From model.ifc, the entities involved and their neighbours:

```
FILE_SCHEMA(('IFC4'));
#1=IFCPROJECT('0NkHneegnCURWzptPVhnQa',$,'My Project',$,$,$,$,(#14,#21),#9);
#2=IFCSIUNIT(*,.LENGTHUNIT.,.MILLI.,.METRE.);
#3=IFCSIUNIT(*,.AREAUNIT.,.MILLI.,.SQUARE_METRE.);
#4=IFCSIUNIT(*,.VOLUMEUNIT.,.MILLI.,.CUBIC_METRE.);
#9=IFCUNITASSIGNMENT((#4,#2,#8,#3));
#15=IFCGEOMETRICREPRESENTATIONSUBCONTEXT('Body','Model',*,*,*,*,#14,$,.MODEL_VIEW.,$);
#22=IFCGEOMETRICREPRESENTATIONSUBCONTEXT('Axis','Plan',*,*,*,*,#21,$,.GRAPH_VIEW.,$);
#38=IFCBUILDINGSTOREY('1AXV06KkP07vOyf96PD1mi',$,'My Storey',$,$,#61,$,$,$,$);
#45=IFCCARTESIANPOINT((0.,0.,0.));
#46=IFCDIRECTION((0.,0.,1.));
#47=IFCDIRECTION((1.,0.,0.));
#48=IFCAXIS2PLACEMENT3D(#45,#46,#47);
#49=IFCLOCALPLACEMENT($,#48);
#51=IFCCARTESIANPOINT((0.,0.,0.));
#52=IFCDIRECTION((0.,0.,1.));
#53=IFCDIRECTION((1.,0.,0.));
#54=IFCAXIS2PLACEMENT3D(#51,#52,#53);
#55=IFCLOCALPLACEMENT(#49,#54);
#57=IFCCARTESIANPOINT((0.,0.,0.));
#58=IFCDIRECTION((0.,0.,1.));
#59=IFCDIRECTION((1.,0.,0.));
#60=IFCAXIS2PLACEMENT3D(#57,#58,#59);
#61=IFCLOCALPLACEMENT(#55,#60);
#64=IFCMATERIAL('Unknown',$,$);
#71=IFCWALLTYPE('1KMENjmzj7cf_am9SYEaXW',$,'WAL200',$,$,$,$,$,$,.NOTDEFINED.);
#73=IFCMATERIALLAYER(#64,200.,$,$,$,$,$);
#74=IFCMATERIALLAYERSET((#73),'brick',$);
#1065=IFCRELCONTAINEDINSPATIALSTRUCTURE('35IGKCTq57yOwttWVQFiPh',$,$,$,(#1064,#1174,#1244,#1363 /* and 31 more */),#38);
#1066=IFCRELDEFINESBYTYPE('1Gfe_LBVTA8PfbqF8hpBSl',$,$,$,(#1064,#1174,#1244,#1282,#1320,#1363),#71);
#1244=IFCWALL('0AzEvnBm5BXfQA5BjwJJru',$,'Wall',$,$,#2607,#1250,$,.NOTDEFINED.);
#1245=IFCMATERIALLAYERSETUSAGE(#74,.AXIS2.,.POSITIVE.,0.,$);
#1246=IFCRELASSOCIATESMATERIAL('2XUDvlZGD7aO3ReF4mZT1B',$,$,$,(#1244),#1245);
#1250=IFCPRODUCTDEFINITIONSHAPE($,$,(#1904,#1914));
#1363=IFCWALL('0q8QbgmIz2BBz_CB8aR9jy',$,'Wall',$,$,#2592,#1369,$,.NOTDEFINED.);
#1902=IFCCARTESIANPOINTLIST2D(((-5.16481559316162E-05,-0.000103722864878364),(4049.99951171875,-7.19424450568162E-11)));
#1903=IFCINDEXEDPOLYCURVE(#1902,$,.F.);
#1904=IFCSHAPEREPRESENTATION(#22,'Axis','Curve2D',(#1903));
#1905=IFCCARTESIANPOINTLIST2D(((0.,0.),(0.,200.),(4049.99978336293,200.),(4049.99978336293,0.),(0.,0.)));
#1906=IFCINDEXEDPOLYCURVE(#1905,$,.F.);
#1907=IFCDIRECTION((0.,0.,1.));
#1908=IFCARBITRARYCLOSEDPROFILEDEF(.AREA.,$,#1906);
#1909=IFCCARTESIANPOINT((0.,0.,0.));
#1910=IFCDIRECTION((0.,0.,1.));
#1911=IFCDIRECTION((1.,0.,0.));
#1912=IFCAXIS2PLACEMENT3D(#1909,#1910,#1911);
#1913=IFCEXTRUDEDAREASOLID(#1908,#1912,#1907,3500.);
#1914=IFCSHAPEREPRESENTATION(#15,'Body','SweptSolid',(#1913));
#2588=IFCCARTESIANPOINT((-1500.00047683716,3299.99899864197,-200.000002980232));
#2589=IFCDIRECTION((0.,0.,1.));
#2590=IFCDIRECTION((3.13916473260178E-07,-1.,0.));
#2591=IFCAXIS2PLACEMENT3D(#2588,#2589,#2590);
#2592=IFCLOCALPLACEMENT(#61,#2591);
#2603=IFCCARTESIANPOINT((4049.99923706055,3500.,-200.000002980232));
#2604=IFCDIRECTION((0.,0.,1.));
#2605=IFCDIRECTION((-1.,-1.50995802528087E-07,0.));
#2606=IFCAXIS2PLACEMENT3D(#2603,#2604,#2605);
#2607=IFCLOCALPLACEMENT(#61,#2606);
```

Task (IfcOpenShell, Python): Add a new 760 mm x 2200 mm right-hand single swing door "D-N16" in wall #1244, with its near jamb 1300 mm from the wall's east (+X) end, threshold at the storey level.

```python
import numpy as np
import ifcopenshell
import ifcopenshell.api.feature
import ifcopenshell.api.geometry
import ifcopenshell.api.root
import ifcopenshell.api.spatial
import ifcopenshell.geom
import ifcopenshell.util.element
import ifcopenshell.util.placement
import ifcopenshell.util.representation
import ifcopenshell.util.shape
import ifcopenshell.util.unit

model = ifcopenshell.open("model.ifc")
unit_scale = ifcopenshell.util.unit.calculate_unit_scale(model)
settings = ifcopenshell.geom.settings()


def volume(element):
    """Net volume in cubic metres, openings subtracted."""
    shape = ifcopenshell.geom.create_shape(settings, element)
    return ifcopenshell.util.shape.get_volume(shape.geometry)


wall = model.by_guid("0AzEvnBm5BXfQA5BjwJJru")
storey = ifcopenshell.util.element.get_container(wall, ifc_class="IfcBuildingStorey")
context = ifcopenshell.util.representation.get_context(model, "Model", "Body", "MODEL_VIEW")
before = volume(wall)

width, height, from_end, sill = 0.76, 2.2, 1.3, 0.0  # metres

# The wall runs along its own X axis, and the end named is its -X end.
wall_shape = ifcopenshell.geom.create_shape(settings, wall)
x, y, z = ifcopenshell.util.shape.get_vertices(wall_shape.geometry).T
start = x.min() + from_end
face, thickness = float(y.min()), float(y.max() - y.min())
wall_matrix = ifcopenshell.util.placement.get_local_placement(wall.ObjectPlacement)
level = ifcopenshell.util.placement.get_local_placement(storey.ObjectPlacement)[2, 3]


def in_wall(x, y):
    """Placement at x, y metres in the wall's axes, at sill height."""
    matrix = wall_matrix.copy()
    matrix[:, 3] = wall_matrix @ np.array([x / unit_scale, y / unit_scale, 0.0, 1.0])
    matrix[2, 3] = level + sill / unit_scale
    return matrix


# Opening: a box that overshoots both wall faces by 50 mm.
opening = ifcopenshell.api.root.create_entity(model, ifc_class="IfcOpeningElement", predefined_type="OPENING")
box = ifcopenshell.api.geometry.add_wall_representation(
    model, context=context, length=width, height=height, thickness=thickness + 0.1
)
ifcopenshell.api.geometry.assign_representation(model, product=opening, representation=box)
ifcopenshell.api.geometry.edit_object_placement(model, product=opening, matrix=in_wall(start, face - 0.05), is_si=False)
ifcopenshell.api.feature.add_feature(model, feature=opening, element=wall)

door = ifcopenshell.api.root.create_entity(model, ifc_class="IfcDoor", name="D-N16", predefined_type="DOOR")
door.OverallWidth, door.OverallHeight = width / unit_scale, height / unit_scale
door.OperationType = "SINGLE_SWING_RIGHT"
body = ifcopenshell.api.geometry.add_door_representation(
    model,
    context=context,
    overall_width=door.OverallWidth,
    overall_height=door.OverallHeight,
    operation_type="SINGLE_SWING_RIGHT",
    lining_properties={"LiningDepth": thickness / unit_scale, "ThresholdDepth": thickness / unit_scale},
)
ifcopenshell.api.geometry.assign_representation(model, product=door, representation=body)
ifcopenshell.api.spatial.assign_container(model, products=[door], relating_structure=storey)
ifcopenshell.api.feature.add_filling(model, opening=opening, element=door)

# The lining spans the wall, so the door starts at the wall face.
ifcopenshell.api.geometry.edit_object_placement(model, product=door, matrix=in_wall(start, face), is_si=False)

after = volume(wall)

print(f"wall volume {before:.3f} -> {after:.3f} m3")

model.write("model_updated.ifc")
```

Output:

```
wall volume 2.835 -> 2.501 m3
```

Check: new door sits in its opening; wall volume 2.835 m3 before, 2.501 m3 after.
